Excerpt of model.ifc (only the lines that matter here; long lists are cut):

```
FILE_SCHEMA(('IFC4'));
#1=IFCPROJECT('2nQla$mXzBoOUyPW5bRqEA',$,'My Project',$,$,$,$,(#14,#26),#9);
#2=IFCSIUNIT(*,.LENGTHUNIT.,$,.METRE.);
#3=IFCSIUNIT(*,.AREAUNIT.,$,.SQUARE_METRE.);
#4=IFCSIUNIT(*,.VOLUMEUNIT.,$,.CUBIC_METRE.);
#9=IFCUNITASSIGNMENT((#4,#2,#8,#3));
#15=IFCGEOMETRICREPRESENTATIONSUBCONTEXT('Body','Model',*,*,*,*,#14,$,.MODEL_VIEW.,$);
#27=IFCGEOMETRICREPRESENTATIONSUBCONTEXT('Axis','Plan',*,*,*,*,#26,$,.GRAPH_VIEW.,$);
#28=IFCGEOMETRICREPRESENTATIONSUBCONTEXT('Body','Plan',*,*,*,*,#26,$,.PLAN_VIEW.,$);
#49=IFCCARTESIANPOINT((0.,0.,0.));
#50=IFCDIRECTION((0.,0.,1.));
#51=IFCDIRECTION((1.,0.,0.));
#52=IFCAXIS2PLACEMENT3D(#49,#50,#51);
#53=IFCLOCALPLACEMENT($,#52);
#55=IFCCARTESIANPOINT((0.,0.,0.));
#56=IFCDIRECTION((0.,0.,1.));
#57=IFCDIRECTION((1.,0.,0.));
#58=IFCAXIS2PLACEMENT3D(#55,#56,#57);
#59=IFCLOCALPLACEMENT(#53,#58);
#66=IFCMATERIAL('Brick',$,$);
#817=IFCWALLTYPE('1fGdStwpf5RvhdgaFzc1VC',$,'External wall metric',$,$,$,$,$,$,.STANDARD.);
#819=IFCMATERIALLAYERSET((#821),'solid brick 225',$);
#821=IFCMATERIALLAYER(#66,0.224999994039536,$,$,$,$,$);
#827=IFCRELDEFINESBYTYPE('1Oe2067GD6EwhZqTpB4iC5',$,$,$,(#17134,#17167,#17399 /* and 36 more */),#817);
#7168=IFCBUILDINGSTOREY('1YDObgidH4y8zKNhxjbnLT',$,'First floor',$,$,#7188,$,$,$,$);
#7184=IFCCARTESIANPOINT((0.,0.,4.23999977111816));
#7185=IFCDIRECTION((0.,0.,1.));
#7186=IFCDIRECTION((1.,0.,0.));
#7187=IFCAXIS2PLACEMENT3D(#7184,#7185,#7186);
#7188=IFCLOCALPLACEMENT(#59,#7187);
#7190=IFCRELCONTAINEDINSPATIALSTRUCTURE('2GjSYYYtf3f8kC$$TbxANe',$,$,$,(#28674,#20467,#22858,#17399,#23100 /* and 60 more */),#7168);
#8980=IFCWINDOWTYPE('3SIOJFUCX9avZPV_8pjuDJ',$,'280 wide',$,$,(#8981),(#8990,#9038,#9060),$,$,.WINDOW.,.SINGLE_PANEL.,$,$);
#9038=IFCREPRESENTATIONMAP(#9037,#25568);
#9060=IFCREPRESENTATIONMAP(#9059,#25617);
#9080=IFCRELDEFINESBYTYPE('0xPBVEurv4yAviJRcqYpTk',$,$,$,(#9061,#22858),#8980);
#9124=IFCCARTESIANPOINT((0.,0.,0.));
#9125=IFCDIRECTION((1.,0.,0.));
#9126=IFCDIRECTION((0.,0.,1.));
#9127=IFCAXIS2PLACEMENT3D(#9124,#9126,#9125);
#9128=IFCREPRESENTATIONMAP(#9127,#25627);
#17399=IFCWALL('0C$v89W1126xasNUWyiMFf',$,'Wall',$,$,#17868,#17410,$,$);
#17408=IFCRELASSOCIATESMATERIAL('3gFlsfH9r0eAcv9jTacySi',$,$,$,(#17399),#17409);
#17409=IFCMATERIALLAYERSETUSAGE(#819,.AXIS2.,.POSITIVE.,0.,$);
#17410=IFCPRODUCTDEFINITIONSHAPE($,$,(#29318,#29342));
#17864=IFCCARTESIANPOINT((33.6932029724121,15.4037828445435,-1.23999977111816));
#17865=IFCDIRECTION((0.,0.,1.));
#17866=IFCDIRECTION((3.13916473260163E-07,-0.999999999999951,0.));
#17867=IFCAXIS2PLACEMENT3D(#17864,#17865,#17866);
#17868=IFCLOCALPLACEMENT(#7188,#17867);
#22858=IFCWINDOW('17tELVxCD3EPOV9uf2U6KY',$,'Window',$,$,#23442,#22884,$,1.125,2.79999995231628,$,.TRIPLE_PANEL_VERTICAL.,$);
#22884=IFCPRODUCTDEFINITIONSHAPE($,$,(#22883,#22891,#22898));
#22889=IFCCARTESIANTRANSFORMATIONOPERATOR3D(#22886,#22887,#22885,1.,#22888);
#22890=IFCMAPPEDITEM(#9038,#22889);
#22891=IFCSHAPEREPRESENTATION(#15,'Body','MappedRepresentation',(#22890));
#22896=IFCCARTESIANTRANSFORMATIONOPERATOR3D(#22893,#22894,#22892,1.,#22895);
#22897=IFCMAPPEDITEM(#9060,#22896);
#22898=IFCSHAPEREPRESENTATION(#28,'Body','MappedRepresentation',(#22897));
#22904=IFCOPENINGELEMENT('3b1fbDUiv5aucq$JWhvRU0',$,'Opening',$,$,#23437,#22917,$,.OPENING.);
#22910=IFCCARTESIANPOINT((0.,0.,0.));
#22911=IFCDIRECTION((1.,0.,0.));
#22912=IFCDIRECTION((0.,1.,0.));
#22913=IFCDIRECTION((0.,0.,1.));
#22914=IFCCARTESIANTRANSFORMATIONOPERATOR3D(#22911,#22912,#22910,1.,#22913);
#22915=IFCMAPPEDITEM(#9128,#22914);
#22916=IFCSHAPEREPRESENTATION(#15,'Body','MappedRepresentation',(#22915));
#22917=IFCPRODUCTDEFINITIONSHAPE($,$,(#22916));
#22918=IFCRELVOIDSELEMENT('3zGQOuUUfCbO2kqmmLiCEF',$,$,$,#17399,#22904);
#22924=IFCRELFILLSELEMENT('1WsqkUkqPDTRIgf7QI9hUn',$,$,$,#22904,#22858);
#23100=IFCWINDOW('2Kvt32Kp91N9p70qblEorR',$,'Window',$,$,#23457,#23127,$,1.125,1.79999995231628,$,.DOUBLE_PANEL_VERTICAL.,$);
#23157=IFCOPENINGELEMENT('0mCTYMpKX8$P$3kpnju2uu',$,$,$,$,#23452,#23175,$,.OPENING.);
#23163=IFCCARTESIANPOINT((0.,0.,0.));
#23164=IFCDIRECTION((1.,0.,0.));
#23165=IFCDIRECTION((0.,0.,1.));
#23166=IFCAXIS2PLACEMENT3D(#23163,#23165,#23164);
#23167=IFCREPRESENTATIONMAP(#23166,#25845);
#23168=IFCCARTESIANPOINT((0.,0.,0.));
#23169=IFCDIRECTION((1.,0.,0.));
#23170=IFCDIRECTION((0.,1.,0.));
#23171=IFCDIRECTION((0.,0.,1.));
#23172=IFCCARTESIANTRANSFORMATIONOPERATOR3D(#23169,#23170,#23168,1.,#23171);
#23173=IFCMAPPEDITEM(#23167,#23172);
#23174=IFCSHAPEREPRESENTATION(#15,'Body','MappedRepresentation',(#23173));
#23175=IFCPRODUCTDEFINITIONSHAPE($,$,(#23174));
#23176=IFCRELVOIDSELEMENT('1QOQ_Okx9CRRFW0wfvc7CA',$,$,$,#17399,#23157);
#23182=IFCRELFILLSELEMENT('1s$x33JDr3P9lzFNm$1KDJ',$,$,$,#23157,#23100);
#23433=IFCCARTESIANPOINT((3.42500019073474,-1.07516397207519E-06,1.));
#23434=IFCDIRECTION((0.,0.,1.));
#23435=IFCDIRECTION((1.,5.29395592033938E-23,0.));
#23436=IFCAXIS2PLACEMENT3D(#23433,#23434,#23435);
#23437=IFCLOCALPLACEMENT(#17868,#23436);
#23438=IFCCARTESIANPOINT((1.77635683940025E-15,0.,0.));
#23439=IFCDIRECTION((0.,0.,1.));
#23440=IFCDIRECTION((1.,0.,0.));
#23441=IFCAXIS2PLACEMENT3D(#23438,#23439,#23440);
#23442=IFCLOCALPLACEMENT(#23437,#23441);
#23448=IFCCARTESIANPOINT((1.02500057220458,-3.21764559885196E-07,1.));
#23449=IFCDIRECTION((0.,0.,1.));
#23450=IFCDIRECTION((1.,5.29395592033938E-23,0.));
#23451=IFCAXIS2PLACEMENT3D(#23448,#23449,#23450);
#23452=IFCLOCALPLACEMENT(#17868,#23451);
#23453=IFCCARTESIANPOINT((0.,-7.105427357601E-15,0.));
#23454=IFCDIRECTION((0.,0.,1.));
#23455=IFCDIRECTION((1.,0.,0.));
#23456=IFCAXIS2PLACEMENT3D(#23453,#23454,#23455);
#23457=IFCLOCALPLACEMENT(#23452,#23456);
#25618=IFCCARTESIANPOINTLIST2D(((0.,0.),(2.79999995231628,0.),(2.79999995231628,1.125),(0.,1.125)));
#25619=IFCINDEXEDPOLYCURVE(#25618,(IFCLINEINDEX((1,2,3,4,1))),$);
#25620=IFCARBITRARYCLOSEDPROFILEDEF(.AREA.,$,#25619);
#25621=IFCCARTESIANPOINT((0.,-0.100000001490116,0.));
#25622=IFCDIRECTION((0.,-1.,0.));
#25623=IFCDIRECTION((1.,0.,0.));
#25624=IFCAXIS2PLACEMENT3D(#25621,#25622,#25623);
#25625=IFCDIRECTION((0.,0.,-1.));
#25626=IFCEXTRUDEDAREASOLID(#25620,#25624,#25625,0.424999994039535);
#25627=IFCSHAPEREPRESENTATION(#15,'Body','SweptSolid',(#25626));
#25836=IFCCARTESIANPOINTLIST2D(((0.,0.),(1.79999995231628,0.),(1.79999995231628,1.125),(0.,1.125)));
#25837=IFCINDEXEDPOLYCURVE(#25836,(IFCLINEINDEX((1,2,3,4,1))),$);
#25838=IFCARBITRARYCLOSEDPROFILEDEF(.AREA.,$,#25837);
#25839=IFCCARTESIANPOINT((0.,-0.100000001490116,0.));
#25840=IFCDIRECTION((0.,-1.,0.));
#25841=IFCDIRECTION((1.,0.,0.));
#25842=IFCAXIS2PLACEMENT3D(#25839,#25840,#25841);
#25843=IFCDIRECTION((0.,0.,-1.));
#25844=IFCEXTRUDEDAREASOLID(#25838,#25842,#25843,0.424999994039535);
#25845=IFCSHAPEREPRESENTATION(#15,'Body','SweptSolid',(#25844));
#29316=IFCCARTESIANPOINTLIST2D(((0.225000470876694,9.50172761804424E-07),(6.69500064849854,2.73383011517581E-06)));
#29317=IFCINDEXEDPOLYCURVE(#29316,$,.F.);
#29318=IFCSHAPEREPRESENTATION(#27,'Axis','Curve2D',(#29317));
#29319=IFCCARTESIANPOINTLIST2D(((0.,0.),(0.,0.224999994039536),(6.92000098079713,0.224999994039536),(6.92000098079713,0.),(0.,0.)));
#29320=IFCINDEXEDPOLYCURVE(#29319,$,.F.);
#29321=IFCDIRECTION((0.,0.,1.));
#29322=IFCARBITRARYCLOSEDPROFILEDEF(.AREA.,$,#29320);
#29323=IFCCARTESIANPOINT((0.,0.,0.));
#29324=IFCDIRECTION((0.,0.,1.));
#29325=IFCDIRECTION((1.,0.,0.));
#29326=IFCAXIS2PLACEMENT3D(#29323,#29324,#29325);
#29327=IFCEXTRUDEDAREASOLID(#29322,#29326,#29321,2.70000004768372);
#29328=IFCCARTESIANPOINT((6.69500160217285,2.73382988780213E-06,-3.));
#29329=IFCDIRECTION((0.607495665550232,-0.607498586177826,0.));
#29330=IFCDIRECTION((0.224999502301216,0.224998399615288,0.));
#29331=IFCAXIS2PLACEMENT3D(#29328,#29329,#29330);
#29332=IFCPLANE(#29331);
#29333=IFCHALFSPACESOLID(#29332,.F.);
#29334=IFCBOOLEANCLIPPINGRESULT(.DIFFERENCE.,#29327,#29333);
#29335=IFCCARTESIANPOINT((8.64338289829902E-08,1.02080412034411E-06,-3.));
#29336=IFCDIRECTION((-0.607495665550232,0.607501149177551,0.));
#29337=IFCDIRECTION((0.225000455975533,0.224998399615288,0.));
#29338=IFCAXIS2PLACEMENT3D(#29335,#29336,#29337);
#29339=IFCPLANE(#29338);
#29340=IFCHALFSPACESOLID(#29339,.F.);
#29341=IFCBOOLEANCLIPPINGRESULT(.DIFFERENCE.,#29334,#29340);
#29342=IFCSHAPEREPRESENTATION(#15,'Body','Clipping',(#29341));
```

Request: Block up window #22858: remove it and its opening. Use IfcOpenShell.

```python
import ifcopenshell
import ifcopenshell.api.feature
import ifcopenshell.api.root
import ifcopenshell.geom
import ifcopenshell.util.shape

model = ifcopenshell.open("model.ifc")
settings = ifcopenshell.geom.settings()


def volume(element):
    """Net volume in cubic metres, openings subtracted."""
    shape = ifcopenshell.geom.create_shape(settings, element)
    return ifcopenshell.util.shape.get_volume(shape.geometry)


window = model.by_guid("17tELVxCD3EPOV9uf2U6KY")
opening = window.FillsVoids[0].RelatingOpeningElement
wall = opening.VoidsElements[0].RelatingBuildingElement
before = volume(wall)

ifcopenshell.api.root.remove_product(model, product=window)
ifcopenshell.api.feature.remove_feature(model, feature=opening)

after = volume(wall)

print(f"wall volume {before:.3f} -> {after:.3f} m3")

model.write("model-out.ifc")
```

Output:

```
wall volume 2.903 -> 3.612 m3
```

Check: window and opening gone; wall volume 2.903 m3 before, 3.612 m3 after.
